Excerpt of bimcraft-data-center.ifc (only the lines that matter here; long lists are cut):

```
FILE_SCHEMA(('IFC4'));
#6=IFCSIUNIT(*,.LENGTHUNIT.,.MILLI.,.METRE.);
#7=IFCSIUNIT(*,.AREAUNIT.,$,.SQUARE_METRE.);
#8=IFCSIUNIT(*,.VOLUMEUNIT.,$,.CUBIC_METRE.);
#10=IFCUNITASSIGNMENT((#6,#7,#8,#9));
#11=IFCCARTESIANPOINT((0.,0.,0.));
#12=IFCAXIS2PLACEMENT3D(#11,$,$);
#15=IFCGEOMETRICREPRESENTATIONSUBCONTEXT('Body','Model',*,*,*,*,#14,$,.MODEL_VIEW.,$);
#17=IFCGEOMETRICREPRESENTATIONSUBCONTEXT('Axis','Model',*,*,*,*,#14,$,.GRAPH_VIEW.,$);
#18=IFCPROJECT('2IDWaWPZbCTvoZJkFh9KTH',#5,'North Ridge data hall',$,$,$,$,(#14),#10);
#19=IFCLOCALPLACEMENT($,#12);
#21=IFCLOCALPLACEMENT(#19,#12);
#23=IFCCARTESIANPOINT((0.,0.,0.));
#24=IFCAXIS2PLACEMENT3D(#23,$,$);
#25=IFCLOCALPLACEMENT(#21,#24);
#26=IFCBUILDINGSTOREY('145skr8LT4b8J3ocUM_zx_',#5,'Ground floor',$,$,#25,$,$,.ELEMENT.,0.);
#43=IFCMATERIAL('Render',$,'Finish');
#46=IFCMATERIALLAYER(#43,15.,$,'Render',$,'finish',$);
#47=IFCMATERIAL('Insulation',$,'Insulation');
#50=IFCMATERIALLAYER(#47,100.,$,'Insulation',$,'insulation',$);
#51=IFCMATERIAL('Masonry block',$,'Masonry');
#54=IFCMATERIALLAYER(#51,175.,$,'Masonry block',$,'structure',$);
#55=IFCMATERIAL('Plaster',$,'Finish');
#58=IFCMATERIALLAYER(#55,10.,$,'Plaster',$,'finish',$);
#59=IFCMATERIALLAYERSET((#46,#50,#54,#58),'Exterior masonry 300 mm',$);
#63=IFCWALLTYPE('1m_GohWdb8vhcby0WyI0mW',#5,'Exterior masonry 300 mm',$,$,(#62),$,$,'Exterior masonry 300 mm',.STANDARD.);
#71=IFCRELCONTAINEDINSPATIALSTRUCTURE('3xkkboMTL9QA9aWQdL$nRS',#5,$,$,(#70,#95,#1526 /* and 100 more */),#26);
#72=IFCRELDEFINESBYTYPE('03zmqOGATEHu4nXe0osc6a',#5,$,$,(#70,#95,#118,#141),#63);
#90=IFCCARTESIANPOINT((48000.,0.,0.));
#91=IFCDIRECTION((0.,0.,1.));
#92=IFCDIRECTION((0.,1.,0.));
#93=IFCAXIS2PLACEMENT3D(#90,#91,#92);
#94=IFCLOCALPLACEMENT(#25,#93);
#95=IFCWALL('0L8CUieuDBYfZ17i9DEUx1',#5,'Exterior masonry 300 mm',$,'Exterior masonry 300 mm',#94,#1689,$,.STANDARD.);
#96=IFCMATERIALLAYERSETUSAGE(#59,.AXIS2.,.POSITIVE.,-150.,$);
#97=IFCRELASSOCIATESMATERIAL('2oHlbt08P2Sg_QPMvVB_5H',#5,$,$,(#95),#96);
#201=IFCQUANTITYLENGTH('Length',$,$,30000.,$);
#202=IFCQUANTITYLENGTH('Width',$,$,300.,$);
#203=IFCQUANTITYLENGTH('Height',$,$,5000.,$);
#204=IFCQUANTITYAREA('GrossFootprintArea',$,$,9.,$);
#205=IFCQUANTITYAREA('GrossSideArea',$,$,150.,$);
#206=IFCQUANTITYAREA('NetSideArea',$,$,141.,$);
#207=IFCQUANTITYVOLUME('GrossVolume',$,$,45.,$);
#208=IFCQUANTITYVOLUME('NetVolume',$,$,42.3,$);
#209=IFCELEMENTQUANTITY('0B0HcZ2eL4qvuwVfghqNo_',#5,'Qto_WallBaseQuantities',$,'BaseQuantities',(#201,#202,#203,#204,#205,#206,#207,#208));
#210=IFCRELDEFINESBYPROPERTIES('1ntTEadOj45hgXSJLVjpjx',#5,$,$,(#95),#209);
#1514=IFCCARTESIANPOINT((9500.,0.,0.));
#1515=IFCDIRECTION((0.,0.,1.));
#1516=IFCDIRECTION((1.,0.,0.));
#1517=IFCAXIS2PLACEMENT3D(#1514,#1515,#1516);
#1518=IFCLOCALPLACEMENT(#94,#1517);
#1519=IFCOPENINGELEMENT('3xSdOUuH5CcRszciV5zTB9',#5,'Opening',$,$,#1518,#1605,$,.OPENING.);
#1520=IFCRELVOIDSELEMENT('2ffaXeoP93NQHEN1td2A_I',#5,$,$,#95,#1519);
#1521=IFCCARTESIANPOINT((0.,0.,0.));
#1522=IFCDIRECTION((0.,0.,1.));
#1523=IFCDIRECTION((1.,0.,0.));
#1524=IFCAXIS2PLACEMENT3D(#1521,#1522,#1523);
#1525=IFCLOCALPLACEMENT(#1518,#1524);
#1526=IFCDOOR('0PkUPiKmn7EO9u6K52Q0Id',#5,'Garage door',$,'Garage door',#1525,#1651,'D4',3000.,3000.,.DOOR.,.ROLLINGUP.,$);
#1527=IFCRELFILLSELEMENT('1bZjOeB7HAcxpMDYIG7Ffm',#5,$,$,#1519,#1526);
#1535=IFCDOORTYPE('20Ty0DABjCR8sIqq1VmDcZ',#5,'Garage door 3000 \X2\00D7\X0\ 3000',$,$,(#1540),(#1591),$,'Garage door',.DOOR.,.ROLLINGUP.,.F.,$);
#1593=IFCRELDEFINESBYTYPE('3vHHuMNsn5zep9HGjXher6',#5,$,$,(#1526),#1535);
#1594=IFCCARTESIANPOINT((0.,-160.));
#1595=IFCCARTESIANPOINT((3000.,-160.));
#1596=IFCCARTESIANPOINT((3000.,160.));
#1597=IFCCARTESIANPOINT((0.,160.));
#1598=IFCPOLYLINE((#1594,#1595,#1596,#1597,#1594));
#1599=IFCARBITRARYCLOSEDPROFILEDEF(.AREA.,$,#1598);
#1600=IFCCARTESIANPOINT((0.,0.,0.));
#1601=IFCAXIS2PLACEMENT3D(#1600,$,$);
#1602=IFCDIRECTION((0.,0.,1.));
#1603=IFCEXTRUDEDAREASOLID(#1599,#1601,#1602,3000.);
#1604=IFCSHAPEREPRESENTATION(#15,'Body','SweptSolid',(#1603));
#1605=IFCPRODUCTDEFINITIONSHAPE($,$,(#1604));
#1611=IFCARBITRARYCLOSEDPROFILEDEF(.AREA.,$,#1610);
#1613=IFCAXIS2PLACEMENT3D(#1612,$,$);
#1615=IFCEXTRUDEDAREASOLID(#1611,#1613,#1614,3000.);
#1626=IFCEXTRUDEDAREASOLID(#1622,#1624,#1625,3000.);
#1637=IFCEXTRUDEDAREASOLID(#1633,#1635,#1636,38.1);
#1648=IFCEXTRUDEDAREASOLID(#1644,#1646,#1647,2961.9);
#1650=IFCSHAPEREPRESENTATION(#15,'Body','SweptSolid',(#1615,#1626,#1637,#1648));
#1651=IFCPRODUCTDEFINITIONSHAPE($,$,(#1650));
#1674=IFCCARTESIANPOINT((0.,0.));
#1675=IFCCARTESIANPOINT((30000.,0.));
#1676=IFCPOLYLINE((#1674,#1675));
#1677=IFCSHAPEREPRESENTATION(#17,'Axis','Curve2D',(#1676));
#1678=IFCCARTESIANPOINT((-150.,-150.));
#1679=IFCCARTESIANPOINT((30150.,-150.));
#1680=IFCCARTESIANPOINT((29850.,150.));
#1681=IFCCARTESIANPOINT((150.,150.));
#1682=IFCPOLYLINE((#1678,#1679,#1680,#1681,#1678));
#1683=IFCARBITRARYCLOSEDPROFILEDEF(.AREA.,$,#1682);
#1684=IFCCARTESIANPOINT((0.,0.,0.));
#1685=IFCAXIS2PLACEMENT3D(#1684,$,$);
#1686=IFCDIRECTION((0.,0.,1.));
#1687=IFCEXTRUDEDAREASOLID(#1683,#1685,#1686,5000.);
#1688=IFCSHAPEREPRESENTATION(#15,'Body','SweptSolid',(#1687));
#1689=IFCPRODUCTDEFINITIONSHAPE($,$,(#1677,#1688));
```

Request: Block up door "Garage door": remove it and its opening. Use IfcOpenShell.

```python
import ifcopenshell
import ifcopenshell.api.feature
import ifcopenshell.api.pset
import ifcopenshell.api.root
import ifcopenshell.geom
import ifcopenshell.util.element
import ifcopenshell.util.shape
import ifcopenshell.util.unit

model = ifcopenshell.open("bimcraft-data-center.ifc")
area_scale = ifcopenshell.util.unit.calculate_unit_scale(model, "AREAUNIT")
volume_scale = ifcopenshell.util.unit.calculate_unit_scale(model, "VOLUMEUNIT")
settings = ifcopenshell.geom.settings()


def volume(element):
    """Net volume in cubic metres, openings subtracted."""
    shape = ifcopenshell.geom.create_shape(settings, element)
    return ifcopenshell.util.shape.get_volume(shape.geometry)


door = model.by_id(1526)
opening = door.FillsVoids[0].RelatingOpeningElement
wall = opening.VoidsElements[0].RelatingBuildingElement
before = volume(wall)

ifcopenshell.api.root.remove_product(model, product=door)
ifcopenshell.api.feature.remove_feature(model, feature=opening)

after = volume(wall)
thickness = 0.3  # wall thickness in metres

# Update the wall's stored quantities.
qto = model.by_id(ifcopenshell.util.element.get_pset(wall, "Qto_WallBaseQuantities", should_inherit=False)["id"])
ifcopenshell.api.pset.edit_qto(model, qto=qto, properties={
    "NetSideArea": after / thickness / area_scale,
    "NetVolume": after / volume_scale,
})

print(f"wall volume {before:.3f} -> {after:.3f} m3")

model.write("bimcraft-data-center-out.ifc")
```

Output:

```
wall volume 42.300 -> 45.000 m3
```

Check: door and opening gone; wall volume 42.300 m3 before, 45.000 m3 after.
